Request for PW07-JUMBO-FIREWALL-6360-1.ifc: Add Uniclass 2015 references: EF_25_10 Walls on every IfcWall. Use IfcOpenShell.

First a look at what the model holds.

```python
import ifcopenshell

model = ifcopenshell.open("PW07-JUMBO-FIREWALL-6360-1.ifc")
print(model.schema)
print("classifications:", [c.Name for c in model.by_type("IfcClassification")])
for ifc_class in ("IfcDoor", "IfcRoof", "IfcStair", "IfcWall", "IfcWindow"):
    print(ifc_class, len(model.by_type(ifc_class)))
```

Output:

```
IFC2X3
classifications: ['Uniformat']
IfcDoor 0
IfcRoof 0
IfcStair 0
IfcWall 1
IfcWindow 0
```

```python
import ifcopenshell
import ifcopenshell.api.classification

model = ifcopenshell.open("PW07-JUMBO-FIREWALL-6360-1.ifc")

# IFC2X3 requires Source and Edition and has no link from the project to the system.
system = model.create_entity("IfcClassification", Source="NBS", Edition="2015", Name="Uniclass 2015")

codes = {
    "IfcWall": ("EF_25_10", "Walls"),
}
for ifc_class, (code, name) in codes.items():
    products = model.by_type(ifc_class)
    ifcopenshell.api.classification.add_reference(
        model, products=products, classification=system, identification=code, name=name
    )
    print(code, len(products))

model.write("PW07-JUMBO-FIREWALL-6360-1_rev.ifc")
```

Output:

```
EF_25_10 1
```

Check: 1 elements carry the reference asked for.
